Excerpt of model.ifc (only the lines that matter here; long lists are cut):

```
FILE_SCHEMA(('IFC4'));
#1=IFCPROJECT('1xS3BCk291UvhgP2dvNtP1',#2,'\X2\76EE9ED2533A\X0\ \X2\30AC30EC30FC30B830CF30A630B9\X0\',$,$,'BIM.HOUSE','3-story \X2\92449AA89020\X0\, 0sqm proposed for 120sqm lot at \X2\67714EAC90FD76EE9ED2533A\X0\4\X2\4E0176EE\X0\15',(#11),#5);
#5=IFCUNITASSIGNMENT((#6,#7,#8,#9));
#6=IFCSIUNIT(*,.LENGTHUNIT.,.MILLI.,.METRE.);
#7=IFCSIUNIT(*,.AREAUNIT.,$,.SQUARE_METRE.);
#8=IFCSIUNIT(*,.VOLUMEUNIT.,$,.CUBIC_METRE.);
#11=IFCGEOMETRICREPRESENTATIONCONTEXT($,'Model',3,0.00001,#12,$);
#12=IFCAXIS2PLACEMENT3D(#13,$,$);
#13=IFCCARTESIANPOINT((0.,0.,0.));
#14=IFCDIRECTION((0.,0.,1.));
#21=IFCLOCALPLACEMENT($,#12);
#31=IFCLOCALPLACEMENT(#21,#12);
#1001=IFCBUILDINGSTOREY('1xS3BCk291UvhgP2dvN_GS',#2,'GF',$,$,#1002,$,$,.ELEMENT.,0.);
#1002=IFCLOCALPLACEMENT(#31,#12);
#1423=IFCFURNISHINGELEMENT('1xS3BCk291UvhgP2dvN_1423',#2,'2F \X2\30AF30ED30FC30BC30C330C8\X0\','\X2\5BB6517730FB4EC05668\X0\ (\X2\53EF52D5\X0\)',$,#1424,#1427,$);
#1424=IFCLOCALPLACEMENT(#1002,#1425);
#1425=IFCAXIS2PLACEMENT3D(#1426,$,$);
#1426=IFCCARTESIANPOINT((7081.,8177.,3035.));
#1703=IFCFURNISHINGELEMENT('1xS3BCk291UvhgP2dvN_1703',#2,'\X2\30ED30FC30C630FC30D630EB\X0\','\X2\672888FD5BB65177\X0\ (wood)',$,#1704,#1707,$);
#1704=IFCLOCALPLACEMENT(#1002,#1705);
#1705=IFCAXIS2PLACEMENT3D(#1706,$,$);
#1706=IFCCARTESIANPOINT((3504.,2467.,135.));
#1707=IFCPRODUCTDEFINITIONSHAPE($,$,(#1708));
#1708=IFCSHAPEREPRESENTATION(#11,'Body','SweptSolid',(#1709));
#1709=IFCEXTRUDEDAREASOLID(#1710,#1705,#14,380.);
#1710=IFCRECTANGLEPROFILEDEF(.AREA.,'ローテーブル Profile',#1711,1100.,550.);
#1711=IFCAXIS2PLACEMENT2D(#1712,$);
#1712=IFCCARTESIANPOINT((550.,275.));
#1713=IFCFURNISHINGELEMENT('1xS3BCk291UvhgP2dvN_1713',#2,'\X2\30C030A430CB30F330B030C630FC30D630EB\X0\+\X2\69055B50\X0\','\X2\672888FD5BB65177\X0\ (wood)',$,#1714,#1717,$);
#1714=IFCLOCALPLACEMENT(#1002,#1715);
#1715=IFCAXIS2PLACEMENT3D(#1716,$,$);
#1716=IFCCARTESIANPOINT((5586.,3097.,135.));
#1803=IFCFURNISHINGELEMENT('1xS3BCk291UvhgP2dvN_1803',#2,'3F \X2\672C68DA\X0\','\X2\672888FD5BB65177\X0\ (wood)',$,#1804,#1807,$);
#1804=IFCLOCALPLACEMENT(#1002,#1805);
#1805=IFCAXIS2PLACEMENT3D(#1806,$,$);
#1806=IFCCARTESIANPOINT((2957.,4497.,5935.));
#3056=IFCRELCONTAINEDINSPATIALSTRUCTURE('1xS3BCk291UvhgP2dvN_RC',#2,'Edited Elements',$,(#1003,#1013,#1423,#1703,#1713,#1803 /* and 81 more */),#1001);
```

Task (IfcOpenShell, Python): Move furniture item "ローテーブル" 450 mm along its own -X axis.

```python
import ifcopenshell
import ifcopenshell.api.geometry
import ifcopenshell.util.placement
import ifcopenshell.util.unit

model = ifcopenshell.open("model.ifc")
unit_scale = ifcopenshell.util.unit.calculate_unit_scale(model)

item = model.by_guid("1xS3BCk291UvhgP2dvN_1703")
matrix = ifcopenshell.util.placement.get_local_placement(item.ObjectPlacement)
matrix[:3, 3] -= matrix[:3, 0] * 0.45 / unit_scale
ifcopenshell.api.geometry.edit_object_placement(model, product=item, matrix=matrix, is_si=False)

print(ifcopenshell.util.placement.get_local_placement(item.ObjectPlacement).round(3) + 0.0)

model.write("model_edited.ifc")
```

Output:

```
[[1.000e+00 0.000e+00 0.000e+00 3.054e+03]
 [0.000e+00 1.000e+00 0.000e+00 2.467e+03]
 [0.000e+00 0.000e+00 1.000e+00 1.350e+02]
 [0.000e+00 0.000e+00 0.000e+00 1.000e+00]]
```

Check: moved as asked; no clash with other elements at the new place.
